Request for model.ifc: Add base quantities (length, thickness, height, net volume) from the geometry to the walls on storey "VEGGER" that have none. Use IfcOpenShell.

First a look at what the model holds.

```python
import ifcopenshell
import ifcopenshell.util.element
import ifcopenshell.util.unit

model = ifcopenshell.open("model.ifc")
print(model.schema)
for unit_type in ("LENGTHUNIT", "AREAUNIT", "VOLUMEUNIT"):
    print(unit_type, ifcopenshell.util.unit.calculate_unit_scale(model, unit_type))
storey = next(s for s in model.by_type("IfcBuildingStorey") if s.Name == "VEGGER")
walls = [e for e in ifcopenshell.util.element.get_decomposition(storey) if e.is_a("IfcWall")]
for e in sorted(walls, key=lambda e: e.id()):
    print(e.id(), e.is_a(), e.Name, list(ifcopenshell.util.element.get_psets(e, qtos_only=True)), sep=" | ")
```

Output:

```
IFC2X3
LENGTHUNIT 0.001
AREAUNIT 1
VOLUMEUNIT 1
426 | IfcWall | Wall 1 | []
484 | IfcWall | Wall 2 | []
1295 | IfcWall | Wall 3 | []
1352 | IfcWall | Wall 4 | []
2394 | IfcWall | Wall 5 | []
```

```python
import ifcopenshell
import ifcopenshell.api.pset
import ifcopenshell.geom
import ifcopenshell.util.element
import ifcopenshell.util.shape
import ifcopenshell.util.unit

model = ifcopenshell.open("model.ifc")
unit_scale = ifcopenshell.util.unit.calculate_unit_scale(model)
volume_scale = ifcopenshell.util.unit.calculate_unit_scale(model, "VOLUMEUNIT")
settings = ifcopenshell.geom.settings()

storey = next(s for s in model.by_type("IfcBuildingStorey") if s.Name == "VEGGER")
walls = [e for e in ifcopenshell.util.element.get_decomposition(storey) if e.is_a("IfcWall")]

for e in sorted(walls, key=lambda e: e.id()):
    if ifcopenshell.util.element.get_psets(e, qtos_only=True, should_inherit=False):
        continue
    # Geometry comes back in metres, in the element's own axes.
    shape = ifcopenshell.geom.create_shape(settings, e)
    values = {
        "Length": ifcopenshell.util.shape.get_x(shape.geometry) / unit_scale,
        "Width": ifcopenshell.util.shape.get_y(shape.geometry) / unit_scale,
        "Height": ifcopenshell.util.shape.get_z(shape.geometry) / unit_scale,
        "NetVolume": ifcopenshell.util.shape.get_volume(shape.geometry) / volume_scale,
    }
    qto = ifcopenshell.api.pset.add_qto(model, product=e, name="BaseQuantities")
    ifcopenshell.api.pset.edit_qto(model, qto=qto, properties=values)
    print(e.id(), {k: round(v, 3) for k, v in values.items()})

model.write("model_edited.ifc")
```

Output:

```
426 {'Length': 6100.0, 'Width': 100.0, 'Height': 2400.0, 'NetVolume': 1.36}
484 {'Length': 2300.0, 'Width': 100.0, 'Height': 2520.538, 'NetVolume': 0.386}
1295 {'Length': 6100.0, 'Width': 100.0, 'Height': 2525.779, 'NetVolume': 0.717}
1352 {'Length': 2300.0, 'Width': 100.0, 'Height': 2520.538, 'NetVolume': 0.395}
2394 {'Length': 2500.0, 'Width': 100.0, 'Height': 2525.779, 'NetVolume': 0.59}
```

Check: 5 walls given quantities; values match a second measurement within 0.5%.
